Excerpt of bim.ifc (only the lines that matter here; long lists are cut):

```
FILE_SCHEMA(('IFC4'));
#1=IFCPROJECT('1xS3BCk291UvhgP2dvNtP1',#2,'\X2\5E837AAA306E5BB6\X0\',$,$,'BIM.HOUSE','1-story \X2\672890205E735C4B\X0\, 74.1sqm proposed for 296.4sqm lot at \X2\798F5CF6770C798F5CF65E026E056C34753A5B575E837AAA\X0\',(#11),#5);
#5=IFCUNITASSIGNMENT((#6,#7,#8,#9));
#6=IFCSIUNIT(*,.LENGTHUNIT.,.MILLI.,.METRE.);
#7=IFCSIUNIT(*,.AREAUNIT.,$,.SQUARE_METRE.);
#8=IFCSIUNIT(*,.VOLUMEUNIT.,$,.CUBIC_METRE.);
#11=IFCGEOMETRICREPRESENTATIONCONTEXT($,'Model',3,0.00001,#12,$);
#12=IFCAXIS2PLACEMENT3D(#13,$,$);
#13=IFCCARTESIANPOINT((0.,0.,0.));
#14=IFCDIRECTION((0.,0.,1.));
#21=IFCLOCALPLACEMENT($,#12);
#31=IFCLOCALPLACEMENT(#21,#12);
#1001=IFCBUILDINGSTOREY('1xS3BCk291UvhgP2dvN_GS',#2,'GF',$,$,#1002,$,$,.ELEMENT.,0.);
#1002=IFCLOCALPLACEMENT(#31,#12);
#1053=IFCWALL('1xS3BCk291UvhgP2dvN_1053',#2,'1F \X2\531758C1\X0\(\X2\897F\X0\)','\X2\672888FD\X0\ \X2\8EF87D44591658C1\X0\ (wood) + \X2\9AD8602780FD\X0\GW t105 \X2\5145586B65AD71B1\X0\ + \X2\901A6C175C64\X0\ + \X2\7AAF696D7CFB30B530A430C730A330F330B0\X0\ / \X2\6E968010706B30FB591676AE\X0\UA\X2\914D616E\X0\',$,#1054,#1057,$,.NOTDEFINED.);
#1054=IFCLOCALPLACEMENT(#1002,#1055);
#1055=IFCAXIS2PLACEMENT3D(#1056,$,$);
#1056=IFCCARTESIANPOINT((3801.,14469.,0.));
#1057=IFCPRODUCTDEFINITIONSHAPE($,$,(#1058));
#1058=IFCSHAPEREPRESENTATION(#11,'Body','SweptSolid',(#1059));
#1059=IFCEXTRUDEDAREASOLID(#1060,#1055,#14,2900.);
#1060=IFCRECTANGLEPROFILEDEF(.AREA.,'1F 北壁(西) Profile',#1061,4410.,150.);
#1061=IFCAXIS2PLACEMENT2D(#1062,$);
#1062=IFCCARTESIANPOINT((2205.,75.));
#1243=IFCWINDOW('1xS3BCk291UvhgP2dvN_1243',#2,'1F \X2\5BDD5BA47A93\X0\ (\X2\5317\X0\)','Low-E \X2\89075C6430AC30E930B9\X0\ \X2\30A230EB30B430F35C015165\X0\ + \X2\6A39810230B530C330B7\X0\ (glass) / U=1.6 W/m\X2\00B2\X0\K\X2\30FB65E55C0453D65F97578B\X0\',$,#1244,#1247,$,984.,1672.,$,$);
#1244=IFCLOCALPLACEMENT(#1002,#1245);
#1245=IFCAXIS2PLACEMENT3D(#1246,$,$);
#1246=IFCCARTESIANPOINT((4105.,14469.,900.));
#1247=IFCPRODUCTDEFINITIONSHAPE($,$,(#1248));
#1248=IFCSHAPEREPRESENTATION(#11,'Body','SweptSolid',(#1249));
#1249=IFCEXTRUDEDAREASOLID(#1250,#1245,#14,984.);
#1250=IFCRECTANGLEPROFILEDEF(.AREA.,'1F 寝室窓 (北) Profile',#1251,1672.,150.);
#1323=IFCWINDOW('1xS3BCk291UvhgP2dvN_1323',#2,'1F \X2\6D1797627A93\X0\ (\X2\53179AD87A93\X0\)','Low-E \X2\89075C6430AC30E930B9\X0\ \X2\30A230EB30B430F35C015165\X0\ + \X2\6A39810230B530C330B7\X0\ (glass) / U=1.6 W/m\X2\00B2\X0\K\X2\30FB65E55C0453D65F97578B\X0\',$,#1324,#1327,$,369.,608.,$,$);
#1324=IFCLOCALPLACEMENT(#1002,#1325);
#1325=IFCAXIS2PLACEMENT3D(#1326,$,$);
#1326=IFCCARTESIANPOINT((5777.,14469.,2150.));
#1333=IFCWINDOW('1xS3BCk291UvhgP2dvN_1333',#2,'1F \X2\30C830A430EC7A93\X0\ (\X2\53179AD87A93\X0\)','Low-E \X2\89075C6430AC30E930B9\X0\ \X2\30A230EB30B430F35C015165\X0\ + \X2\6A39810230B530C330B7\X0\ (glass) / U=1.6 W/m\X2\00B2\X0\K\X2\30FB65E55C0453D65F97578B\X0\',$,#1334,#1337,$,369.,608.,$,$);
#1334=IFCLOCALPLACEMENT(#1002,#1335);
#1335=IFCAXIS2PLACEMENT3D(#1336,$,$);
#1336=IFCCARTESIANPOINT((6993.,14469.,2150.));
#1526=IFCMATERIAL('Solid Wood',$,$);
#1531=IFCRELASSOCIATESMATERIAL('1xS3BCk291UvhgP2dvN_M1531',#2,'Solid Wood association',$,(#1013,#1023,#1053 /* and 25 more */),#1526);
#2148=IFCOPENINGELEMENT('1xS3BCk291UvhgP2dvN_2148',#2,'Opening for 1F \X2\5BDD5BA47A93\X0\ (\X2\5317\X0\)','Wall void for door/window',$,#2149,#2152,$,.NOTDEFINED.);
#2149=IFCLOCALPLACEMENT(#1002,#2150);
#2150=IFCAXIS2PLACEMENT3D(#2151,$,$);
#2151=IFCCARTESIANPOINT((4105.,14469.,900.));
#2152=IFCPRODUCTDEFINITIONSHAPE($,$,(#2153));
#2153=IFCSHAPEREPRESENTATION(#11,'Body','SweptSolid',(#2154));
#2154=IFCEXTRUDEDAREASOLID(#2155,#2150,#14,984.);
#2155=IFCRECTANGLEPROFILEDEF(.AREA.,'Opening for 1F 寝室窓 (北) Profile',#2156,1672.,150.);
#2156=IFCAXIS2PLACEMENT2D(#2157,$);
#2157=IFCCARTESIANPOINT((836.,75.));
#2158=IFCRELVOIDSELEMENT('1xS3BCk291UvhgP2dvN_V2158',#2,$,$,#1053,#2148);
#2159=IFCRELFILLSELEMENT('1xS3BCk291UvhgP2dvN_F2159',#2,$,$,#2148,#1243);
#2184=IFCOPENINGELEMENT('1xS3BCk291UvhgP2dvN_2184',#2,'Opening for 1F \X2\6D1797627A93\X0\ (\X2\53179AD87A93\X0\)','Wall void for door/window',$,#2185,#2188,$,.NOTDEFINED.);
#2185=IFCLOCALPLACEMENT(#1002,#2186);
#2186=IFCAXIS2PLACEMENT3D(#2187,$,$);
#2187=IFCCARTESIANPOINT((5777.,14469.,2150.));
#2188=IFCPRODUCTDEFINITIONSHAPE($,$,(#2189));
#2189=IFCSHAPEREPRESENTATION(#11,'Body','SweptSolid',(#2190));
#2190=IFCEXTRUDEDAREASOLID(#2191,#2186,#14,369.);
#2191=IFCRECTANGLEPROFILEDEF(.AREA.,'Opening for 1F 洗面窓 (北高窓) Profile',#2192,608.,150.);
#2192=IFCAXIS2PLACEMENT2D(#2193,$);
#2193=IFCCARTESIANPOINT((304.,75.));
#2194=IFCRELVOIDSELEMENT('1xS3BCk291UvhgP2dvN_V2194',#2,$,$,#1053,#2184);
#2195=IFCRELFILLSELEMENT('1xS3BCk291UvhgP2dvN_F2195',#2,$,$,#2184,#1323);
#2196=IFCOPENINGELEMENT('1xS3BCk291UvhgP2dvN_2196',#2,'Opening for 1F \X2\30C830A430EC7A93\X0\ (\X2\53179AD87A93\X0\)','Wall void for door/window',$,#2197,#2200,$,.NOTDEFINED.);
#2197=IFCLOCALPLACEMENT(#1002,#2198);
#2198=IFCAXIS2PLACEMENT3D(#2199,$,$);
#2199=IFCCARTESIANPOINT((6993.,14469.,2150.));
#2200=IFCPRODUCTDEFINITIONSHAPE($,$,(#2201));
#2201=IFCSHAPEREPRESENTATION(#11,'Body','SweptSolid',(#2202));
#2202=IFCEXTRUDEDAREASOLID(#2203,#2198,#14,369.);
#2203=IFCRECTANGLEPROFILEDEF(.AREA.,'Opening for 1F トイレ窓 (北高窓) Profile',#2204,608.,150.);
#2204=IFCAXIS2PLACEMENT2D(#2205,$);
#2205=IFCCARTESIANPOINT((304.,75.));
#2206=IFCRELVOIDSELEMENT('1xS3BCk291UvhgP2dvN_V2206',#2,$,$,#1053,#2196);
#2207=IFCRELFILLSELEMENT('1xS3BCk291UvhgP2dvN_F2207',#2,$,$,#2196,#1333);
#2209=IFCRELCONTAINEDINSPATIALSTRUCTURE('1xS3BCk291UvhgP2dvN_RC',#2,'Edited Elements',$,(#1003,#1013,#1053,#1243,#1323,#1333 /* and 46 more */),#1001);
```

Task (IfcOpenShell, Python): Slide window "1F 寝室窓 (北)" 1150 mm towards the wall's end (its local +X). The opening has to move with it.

```python
import ifcopenshell
import ifcopenshell.api.geometry
import ifcopenshell.util.placement
import ifcopenshell.util.unit

model = ifcopenshell.open("bim.ifc")
unit_scale = ifcopenshell.util.unit.calculate_unit_scale(model)

window = model.by_guid("1xS3BCk291UvhgP2dvN_1243")
opening = window.FillsVoids[0].RelatingOpeningElement
wall = opening.VoidsElements[0].RelatingBuildingElement

wall_matrix = ifcopenshell.util.placement.get_local_placement(wall.ObjectPlacement)
shift = wall_matrix[:3, 0] * 1.15 / unit_scale
before = ifcopenshell.util.placement.get_local_placement(window.ObjectPlacement)[:3, 3].copy()

# The window is not placed relative to its opening, so move both.
for product in (opening, window):
    matrix = ifcopenshell.util.placement.get_local_placement(product.ObjectPlacement)
    matrix[:3, 3] += shift
    ifcopenshell.api.geometry.edit_object_placement(model, product=product, matrix=matrix, is_si=False)

after = ifcopenshell.util.placement.get_local_placement(window.ObjectPlacement)[:3, 3]
print("window moved by", (after - before).round(3) + 0.0)

model.write("bim-out.ifc")
```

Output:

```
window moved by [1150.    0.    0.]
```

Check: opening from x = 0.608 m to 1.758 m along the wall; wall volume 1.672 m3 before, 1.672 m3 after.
